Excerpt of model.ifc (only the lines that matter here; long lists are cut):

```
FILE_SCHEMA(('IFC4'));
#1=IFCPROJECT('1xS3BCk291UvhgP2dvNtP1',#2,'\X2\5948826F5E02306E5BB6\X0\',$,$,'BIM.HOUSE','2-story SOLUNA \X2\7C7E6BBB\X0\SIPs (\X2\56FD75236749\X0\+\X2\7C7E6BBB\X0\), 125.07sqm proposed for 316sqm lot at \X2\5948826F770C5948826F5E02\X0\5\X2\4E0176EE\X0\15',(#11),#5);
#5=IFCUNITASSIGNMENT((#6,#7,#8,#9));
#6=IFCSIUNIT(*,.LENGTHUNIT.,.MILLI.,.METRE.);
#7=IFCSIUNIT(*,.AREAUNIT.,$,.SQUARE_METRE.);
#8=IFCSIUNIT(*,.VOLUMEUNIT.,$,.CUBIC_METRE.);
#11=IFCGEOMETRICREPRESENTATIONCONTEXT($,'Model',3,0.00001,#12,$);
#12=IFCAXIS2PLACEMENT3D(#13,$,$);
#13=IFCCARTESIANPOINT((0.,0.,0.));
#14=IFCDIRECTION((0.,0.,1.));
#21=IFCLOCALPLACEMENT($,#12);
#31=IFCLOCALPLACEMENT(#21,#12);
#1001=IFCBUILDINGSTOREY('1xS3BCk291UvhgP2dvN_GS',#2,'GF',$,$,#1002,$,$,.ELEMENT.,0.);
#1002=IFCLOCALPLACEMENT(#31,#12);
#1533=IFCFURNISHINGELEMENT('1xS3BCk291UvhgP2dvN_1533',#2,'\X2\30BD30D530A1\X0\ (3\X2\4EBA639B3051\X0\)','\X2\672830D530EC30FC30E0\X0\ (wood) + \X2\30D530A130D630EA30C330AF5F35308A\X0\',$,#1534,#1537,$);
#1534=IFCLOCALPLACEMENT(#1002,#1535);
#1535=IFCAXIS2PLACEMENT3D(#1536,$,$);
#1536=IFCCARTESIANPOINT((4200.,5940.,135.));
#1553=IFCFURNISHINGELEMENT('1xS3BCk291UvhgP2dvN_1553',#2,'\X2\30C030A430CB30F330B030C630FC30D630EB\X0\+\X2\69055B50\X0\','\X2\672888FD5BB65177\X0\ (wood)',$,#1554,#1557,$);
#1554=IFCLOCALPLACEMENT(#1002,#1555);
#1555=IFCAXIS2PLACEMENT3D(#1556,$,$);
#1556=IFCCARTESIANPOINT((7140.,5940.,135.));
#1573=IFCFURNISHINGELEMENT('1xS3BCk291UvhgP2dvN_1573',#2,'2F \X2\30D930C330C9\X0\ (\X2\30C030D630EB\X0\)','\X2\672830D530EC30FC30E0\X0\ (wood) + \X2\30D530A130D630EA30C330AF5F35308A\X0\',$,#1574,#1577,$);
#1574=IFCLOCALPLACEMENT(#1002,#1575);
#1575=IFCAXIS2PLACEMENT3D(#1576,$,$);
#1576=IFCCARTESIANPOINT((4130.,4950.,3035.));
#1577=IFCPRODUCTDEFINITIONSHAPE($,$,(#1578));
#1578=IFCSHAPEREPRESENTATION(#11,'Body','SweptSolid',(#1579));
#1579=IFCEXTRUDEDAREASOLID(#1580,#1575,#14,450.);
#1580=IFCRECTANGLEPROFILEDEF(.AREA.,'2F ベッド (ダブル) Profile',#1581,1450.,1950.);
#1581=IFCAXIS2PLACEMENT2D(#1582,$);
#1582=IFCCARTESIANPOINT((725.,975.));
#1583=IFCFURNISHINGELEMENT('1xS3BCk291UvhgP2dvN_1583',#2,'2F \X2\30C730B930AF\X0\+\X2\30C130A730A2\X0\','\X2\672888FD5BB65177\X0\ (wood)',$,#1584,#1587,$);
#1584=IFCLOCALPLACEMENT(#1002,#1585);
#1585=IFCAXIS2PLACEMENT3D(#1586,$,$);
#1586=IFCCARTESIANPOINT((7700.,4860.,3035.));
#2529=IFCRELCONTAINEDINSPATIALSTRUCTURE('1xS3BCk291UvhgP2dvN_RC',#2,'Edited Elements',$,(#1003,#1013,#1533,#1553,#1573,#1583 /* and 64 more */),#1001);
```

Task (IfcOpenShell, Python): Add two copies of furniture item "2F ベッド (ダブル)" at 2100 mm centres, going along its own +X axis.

```python
import ifcopenshell
import ifcopenshell.api.geometry
import ifcopenshell.api.root
import ifcopenshell.util.element
import ifcopenshell.util.placement
import ifcopenshell.util.unit

model = ifcopenshell.open("model.ifc")
unit_scale = ifcopenshell.util.unit.calculate_unit_scale(model)


def reuse_history(source, copy):
    """copy_class also copies each property set's owner history, people and application; keep the originals."""
    for rel in copy.IsDefinedBy:
        if rel.is_a("IfcRelDefinesByProperties") and (history := rel.RelatingPropertyDefinition.OwnerHistory):
            rel.RelatingPropertyDefinition.OwnerHistory = source.OwnerHistory
            ifcopenshell.util.element.remove_deep2(model, history)


source = model.by_guid("1xS3BCk291UvhgP2dvN_1573")
base = ifcopenshell.util.placement.get_local_placement(source.ObjectPlacement)
step = base[:3, 0] * 2.1 / unit_scale

for i in range(1, 3):
    copy = ifcopenshell.api.root.copy_class(model, product=source)
    copy.Representation = ifcopenshell.util.element.copy_deep(
        model, source.Representation, exclude=["IfcGeometricRepresentationContext", "IfcRepresentationMap"]
    )
    reuse_history(source, copy)
    matrix = base.copy()
    matrix[:3, 3] += i * step
    print("added at", matrix[:3, 3].round(3) + 0.0)
    ifcopenshell.api.geometry.edit_object_placement(model, product=copy, matrix=matrix, is_si=False)

model.write("model-out.ifc")
```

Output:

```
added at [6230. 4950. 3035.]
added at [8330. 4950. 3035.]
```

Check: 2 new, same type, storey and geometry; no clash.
